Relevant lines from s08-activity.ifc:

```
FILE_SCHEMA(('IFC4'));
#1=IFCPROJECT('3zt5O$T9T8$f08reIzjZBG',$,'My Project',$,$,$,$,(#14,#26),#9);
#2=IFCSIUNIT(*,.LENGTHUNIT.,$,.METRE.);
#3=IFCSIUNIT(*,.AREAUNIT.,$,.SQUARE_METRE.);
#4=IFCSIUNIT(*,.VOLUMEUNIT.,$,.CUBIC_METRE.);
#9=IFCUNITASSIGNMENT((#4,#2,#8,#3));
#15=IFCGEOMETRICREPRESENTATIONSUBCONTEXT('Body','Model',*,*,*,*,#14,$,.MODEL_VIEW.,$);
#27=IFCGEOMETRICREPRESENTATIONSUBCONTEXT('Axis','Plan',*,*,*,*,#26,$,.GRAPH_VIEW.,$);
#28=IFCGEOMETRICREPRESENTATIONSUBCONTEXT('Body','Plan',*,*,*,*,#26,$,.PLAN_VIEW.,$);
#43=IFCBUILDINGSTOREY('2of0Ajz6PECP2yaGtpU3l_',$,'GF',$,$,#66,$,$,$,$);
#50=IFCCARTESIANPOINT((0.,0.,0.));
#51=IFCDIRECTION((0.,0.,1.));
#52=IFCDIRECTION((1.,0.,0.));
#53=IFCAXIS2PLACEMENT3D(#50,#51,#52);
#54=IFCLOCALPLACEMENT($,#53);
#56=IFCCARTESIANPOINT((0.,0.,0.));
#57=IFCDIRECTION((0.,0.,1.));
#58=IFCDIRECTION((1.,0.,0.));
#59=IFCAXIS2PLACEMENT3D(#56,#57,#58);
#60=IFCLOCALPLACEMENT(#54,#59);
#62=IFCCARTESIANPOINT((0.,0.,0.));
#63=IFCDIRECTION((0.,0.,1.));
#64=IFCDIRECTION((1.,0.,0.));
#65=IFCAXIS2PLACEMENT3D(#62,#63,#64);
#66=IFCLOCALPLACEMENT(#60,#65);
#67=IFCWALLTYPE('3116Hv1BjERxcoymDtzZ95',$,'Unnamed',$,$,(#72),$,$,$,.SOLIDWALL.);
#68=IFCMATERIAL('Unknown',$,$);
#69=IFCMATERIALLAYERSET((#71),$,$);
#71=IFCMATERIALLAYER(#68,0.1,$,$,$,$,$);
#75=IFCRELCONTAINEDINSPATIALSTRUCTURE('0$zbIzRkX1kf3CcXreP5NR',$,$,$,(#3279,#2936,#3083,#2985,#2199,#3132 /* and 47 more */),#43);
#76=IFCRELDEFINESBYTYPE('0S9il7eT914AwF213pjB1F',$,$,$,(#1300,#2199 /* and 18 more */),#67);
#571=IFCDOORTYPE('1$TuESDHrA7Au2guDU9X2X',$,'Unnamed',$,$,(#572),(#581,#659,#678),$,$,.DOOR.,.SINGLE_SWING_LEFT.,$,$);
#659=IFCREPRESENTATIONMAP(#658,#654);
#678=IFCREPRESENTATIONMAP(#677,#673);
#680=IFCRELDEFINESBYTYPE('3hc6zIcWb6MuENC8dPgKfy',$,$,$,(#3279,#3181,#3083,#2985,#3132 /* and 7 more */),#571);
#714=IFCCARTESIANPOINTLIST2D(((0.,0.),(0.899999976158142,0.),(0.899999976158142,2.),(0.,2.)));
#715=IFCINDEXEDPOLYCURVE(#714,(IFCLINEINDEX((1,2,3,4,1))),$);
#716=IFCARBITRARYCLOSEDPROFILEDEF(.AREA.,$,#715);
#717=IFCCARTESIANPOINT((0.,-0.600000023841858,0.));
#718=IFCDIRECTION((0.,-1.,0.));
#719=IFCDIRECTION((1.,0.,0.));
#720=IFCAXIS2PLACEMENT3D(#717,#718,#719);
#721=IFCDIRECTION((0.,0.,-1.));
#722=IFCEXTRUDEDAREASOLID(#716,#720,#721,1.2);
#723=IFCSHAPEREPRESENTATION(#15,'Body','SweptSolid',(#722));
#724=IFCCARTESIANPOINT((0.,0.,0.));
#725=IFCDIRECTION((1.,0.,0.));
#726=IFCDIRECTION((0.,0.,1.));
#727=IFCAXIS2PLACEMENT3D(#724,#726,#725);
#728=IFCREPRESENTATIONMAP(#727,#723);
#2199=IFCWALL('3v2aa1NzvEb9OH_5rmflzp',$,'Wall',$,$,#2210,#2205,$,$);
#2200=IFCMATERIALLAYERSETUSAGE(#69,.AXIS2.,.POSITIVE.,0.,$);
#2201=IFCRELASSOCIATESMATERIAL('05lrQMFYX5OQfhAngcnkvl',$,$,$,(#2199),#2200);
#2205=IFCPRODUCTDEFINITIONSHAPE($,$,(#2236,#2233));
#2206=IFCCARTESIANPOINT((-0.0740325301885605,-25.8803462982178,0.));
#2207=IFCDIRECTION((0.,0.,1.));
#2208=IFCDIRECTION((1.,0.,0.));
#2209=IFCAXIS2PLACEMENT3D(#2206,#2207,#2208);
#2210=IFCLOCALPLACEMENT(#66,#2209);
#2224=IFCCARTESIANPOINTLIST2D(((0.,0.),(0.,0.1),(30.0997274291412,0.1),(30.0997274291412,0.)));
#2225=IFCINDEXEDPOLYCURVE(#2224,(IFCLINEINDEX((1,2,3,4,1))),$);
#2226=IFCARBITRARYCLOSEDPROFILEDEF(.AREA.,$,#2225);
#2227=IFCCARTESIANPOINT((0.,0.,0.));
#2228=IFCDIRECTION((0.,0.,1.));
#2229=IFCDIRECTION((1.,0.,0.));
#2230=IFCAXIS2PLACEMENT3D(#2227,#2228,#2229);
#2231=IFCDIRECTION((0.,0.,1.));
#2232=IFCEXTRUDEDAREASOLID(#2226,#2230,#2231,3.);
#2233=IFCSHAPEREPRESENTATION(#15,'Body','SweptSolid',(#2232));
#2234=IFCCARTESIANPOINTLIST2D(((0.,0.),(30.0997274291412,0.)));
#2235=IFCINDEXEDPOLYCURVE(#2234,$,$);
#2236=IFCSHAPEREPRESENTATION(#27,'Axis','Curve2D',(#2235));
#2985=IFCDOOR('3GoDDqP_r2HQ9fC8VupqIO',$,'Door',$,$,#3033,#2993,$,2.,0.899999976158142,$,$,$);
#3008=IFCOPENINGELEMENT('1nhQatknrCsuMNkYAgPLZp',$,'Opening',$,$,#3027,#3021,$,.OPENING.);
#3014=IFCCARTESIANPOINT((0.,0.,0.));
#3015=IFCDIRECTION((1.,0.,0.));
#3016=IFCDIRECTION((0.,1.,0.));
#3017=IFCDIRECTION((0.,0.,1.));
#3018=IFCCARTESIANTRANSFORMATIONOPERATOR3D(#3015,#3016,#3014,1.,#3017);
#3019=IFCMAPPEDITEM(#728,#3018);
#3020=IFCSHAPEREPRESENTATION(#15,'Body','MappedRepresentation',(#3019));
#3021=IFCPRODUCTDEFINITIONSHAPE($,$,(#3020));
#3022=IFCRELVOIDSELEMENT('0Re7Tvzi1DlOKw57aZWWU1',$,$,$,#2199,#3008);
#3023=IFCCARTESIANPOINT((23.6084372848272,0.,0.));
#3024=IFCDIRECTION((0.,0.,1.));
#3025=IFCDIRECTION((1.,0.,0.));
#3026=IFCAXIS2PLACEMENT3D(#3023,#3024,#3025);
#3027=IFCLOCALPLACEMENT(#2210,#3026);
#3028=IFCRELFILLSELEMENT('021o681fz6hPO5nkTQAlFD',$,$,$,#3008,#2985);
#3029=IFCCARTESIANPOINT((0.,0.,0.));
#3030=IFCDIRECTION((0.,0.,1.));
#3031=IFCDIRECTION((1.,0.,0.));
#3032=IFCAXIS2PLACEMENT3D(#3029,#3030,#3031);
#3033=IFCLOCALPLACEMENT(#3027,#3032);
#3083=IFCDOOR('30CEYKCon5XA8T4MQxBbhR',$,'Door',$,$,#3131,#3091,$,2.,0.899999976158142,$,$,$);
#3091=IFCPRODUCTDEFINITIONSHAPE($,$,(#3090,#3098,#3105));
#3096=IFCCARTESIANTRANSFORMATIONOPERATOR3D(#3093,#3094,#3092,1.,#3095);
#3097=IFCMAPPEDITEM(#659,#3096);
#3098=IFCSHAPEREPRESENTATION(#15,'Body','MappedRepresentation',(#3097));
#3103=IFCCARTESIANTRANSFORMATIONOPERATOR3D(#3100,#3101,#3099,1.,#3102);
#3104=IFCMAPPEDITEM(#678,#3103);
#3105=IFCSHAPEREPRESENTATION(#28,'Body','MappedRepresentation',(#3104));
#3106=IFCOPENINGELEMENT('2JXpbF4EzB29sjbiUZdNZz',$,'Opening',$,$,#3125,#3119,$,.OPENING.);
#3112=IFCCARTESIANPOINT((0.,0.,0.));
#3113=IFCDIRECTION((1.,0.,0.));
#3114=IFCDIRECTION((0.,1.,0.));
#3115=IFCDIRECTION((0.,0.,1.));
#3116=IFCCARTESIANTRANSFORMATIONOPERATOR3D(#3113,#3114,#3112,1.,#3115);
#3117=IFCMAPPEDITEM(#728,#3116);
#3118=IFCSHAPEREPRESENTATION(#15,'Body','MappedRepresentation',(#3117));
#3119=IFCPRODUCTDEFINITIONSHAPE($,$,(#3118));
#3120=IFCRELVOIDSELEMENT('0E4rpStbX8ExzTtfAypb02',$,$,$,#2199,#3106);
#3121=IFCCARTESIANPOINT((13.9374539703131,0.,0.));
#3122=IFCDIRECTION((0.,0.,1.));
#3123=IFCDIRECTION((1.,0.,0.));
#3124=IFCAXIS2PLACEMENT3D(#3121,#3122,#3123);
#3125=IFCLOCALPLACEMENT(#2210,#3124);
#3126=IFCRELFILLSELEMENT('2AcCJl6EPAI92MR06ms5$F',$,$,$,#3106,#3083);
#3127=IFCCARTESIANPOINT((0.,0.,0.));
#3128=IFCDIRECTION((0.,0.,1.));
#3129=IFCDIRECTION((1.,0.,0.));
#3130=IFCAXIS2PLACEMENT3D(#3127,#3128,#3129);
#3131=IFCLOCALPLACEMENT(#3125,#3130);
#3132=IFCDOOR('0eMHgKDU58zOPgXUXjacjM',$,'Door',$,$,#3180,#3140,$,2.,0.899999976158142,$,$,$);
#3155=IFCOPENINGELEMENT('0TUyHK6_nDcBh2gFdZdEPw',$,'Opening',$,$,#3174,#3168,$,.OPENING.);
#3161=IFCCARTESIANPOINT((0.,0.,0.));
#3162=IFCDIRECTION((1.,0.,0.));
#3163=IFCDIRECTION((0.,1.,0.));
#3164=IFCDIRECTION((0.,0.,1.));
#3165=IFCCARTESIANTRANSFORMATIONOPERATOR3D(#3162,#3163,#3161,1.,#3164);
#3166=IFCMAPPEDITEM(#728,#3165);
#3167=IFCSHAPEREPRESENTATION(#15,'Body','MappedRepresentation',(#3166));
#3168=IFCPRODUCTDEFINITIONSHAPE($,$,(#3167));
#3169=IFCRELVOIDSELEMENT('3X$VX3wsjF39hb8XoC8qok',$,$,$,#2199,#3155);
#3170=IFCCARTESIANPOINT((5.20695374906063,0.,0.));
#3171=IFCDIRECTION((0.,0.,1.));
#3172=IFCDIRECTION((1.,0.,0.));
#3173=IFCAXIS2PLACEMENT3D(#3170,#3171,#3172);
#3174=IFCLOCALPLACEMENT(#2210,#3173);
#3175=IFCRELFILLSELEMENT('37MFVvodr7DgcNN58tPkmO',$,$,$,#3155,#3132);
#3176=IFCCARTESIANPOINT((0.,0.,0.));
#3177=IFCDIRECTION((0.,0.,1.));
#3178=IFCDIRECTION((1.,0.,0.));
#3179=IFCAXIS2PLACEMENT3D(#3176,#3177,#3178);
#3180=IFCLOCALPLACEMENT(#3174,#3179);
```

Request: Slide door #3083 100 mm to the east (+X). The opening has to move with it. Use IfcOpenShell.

```python
import ifcopenshell
import ifcopenshell.api.geometry
import ifcopenshell.util.placement

model = ifcopenshell.open("s08-activity.ifc")

door = model.by_guid("30CEYKCon5XA8T4MQxBbhR")
opening = door.FillsVoids[0].RelatingOpeningElement
wall = opening.VoidsElements[0].RelatingBuildingElement

wall_matrix = ifcopenshell.util.placement.get_local_placement(wall.ObjectPlacement)
shift = wall_matrix[:3, 0] * 0.1
before = ifcopenshell.util.placement.get_local_placement(door.ObjectPlacement)[:3, 3].copy()

# The door is placed relative to its opening, so it follows when the opening moves.
matrix = ifcopenshell.util.placement.get_local_placement(opening.ObjectPlacement)
matrix[:3, 3] += shift
ifcopenshell.api.geometry.edit_object_placement(
    model, product=opening, matrix=matrix, is_si=False, should_transform_children=True
)

after = ifcopenshell.util.placement.get_local_placement(door.ObjectPlacement)[:3, 3]
print("door moved by", (after - before).round(3) + 0.0)

model.write("s08-activity_edited.ifc")
```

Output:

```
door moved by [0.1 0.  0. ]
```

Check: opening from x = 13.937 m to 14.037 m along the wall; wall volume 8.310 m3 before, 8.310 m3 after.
